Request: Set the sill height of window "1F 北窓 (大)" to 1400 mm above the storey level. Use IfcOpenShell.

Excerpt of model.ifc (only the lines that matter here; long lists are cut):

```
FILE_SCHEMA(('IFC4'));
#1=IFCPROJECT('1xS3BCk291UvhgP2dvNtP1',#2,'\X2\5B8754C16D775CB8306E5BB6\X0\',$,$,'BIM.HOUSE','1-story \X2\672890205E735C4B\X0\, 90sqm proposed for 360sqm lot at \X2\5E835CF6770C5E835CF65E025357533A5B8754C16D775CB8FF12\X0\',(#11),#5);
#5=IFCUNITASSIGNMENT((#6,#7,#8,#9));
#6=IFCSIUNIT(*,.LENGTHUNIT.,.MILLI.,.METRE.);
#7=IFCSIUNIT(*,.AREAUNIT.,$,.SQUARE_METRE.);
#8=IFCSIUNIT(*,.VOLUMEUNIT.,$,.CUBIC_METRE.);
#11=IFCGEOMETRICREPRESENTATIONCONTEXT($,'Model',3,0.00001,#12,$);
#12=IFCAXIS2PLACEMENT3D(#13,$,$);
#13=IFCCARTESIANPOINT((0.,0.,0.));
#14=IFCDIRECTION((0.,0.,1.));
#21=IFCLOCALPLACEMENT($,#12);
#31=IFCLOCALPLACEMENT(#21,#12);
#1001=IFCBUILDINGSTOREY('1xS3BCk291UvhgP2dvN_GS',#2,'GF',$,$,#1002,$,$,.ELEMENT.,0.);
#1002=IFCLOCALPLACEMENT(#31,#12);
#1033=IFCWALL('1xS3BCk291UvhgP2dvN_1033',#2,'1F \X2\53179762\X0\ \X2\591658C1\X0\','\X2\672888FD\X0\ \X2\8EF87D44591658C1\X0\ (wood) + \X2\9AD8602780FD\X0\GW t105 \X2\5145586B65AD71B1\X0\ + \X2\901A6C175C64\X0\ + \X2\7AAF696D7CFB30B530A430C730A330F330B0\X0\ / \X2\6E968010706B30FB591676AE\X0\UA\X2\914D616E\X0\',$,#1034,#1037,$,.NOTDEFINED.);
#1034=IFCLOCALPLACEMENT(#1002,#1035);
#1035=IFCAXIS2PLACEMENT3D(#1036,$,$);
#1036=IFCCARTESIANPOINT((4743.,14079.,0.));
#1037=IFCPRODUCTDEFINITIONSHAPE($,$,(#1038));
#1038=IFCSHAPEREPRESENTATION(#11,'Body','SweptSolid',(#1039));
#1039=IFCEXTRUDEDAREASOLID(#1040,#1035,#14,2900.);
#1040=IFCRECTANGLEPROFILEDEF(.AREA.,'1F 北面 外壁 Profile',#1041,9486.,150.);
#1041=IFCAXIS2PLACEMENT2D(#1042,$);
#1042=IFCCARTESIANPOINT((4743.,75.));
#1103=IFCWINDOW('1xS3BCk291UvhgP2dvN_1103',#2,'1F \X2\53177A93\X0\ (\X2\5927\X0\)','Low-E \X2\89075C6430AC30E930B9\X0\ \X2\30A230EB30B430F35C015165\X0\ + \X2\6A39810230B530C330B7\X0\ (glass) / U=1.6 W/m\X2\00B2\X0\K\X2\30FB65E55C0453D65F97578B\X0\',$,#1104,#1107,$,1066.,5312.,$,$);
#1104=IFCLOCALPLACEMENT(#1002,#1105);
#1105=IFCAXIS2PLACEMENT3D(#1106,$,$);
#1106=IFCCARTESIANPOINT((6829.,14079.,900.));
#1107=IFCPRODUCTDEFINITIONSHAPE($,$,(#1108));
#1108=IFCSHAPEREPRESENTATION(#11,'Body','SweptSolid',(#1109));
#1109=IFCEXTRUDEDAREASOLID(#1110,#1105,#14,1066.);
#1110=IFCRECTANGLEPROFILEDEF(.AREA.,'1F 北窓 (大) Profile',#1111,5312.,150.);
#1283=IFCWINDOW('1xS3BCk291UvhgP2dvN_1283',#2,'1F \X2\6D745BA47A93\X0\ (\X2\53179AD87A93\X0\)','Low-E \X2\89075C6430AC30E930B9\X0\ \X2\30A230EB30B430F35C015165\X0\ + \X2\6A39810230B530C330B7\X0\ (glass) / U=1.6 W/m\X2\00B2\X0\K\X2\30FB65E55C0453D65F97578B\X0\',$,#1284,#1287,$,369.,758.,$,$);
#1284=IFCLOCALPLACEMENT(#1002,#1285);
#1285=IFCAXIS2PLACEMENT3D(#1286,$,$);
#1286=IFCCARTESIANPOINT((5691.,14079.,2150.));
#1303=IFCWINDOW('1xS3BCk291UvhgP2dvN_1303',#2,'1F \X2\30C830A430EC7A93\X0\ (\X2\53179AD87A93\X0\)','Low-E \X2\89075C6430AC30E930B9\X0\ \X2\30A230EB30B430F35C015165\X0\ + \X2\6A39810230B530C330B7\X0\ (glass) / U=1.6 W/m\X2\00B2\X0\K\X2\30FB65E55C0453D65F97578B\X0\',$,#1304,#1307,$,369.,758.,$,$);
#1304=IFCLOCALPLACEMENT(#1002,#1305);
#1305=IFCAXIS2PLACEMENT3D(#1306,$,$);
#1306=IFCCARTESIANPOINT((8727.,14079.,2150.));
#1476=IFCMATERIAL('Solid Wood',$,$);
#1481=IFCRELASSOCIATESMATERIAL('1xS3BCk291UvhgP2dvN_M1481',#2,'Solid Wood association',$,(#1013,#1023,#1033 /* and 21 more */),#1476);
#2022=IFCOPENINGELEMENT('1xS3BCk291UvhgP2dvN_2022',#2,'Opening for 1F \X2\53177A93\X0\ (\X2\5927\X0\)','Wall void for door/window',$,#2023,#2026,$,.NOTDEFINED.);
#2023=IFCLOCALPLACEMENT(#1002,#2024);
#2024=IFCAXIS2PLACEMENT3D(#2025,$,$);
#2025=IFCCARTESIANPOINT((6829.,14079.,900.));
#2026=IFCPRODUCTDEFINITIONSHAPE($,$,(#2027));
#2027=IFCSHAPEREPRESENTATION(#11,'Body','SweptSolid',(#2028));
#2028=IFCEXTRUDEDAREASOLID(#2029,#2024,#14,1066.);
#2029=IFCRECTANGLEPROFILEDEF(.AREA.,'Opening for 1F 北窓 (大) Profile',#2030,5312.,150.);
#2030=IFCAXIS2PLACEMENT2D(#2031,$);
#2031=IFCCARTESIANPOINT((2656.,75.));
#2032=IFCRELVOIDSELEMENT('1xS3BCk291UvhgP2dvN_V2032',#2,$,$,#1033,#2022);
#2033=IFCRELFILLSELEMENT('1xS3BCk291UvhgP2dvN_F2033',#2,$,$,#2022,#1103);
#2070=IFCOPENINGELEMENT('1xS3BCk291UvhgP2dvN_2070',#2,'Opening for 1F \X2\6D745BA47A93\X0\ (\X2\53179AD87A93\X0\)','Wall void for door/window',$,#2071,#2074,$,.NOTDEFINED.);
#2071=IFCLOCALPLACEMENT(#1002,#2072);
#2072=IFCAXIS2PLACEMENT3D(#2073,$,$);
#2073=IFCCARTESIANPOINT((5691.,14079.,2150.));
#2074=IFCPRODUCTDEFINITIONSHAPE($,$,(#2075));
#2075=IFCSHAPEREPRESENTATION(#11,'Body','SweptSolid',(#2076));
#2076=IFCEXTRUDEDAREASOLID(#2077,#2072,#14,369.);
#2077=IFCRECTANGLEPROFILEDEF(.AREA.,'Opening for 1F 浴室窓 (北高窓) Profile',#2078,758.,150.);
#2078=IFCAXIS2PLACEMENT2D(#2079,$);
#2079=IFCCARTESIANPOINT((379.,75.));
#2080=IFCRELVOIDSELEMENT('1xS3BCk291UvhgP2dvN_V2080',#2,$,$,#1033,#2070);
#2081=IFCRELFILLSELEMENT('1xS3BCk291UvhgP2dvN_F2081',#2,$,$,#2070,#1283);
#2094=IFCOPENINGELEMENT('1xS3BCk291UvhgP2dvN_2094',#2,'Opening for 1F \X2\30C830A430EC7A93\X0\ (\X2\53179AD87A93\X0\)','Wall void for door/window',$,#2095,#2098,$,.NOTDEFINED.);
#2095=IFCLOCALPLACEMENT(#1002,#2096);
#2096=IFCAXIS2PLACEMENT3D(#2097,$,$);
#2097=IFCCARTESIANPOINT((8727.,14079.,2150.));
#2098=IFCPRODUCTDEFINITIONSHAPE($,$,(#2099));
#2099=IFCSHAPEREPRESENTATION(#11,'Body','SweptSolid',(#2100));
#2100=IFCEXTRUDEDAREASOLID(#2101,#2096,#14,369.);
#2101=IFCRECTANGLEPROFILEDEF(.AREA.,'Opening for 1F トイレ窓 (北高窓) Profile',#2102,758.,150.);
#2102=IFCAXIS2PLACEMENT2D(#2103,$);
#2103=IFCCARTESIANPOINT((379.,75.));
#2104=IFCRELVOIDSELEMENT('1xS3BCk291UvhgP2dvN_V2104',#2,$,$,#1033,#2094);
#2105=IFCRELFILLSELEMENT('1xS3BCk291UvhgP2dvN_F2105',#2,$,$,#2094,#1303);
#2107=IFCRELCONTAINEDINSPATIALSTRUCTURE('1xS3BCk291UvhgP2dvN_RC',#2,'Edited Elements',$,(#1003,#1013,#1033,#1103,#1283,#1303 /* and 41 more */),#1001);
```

```python
import numpy as np
import ifcopenshell
import ifcopenshell.api.geometry
import ifcopenshell.geom
import ifcopenshell.util.element
import ifcopenshell.util.placement
import ifcopenshell.util.shape
import ifcopenshell.util.unit

model = ifcopenshell.open("model.ifc")
unit_scale = ifcopenshell.util.unit.calculate_unit_scale(model)

window = model.by_id(1103)
opening = window.FillsVoids[0].RelatingOpeningElement
storey = ifcopenshell.util.element.get_container(window, ifc_class="IfcBuildingStorey")
level = ifcopenshell.util.placement.get_local_placement(storey.ObjectPlacement)[2, 3]

# The opening's origin need not be at the sill, so measure its lowest point.
shape = ifcopenshell.geom.create_shape(ifcopenshell.geom.settings(), opening)
bottom = ifcopenshell.util.shape.get_shape_bottom_elevation(shape, shape.geometry) / unit_scale
dz = level + 1.4 / unit_scale - bottom

shift = np.array([0.0, 0.0, dz])
# The window is not placed relative to its opening, so move both.
for product in (opening, window):
    matrix = ifcopenshell.util.placement.get_local_placement(product.ObjectPlacement)
    matrix[:3, 3] += shift
    ifcopenshell.api.geometry.edit_object_placement(model, product=product, matrix=matrix, is_si=False)

print(f"moved by {dz * unit_scale:+.3f} m")

model.write("model_rev.ifc")
```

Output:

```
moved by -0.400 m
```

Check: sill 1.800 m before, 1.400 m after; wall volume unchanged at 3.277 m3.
